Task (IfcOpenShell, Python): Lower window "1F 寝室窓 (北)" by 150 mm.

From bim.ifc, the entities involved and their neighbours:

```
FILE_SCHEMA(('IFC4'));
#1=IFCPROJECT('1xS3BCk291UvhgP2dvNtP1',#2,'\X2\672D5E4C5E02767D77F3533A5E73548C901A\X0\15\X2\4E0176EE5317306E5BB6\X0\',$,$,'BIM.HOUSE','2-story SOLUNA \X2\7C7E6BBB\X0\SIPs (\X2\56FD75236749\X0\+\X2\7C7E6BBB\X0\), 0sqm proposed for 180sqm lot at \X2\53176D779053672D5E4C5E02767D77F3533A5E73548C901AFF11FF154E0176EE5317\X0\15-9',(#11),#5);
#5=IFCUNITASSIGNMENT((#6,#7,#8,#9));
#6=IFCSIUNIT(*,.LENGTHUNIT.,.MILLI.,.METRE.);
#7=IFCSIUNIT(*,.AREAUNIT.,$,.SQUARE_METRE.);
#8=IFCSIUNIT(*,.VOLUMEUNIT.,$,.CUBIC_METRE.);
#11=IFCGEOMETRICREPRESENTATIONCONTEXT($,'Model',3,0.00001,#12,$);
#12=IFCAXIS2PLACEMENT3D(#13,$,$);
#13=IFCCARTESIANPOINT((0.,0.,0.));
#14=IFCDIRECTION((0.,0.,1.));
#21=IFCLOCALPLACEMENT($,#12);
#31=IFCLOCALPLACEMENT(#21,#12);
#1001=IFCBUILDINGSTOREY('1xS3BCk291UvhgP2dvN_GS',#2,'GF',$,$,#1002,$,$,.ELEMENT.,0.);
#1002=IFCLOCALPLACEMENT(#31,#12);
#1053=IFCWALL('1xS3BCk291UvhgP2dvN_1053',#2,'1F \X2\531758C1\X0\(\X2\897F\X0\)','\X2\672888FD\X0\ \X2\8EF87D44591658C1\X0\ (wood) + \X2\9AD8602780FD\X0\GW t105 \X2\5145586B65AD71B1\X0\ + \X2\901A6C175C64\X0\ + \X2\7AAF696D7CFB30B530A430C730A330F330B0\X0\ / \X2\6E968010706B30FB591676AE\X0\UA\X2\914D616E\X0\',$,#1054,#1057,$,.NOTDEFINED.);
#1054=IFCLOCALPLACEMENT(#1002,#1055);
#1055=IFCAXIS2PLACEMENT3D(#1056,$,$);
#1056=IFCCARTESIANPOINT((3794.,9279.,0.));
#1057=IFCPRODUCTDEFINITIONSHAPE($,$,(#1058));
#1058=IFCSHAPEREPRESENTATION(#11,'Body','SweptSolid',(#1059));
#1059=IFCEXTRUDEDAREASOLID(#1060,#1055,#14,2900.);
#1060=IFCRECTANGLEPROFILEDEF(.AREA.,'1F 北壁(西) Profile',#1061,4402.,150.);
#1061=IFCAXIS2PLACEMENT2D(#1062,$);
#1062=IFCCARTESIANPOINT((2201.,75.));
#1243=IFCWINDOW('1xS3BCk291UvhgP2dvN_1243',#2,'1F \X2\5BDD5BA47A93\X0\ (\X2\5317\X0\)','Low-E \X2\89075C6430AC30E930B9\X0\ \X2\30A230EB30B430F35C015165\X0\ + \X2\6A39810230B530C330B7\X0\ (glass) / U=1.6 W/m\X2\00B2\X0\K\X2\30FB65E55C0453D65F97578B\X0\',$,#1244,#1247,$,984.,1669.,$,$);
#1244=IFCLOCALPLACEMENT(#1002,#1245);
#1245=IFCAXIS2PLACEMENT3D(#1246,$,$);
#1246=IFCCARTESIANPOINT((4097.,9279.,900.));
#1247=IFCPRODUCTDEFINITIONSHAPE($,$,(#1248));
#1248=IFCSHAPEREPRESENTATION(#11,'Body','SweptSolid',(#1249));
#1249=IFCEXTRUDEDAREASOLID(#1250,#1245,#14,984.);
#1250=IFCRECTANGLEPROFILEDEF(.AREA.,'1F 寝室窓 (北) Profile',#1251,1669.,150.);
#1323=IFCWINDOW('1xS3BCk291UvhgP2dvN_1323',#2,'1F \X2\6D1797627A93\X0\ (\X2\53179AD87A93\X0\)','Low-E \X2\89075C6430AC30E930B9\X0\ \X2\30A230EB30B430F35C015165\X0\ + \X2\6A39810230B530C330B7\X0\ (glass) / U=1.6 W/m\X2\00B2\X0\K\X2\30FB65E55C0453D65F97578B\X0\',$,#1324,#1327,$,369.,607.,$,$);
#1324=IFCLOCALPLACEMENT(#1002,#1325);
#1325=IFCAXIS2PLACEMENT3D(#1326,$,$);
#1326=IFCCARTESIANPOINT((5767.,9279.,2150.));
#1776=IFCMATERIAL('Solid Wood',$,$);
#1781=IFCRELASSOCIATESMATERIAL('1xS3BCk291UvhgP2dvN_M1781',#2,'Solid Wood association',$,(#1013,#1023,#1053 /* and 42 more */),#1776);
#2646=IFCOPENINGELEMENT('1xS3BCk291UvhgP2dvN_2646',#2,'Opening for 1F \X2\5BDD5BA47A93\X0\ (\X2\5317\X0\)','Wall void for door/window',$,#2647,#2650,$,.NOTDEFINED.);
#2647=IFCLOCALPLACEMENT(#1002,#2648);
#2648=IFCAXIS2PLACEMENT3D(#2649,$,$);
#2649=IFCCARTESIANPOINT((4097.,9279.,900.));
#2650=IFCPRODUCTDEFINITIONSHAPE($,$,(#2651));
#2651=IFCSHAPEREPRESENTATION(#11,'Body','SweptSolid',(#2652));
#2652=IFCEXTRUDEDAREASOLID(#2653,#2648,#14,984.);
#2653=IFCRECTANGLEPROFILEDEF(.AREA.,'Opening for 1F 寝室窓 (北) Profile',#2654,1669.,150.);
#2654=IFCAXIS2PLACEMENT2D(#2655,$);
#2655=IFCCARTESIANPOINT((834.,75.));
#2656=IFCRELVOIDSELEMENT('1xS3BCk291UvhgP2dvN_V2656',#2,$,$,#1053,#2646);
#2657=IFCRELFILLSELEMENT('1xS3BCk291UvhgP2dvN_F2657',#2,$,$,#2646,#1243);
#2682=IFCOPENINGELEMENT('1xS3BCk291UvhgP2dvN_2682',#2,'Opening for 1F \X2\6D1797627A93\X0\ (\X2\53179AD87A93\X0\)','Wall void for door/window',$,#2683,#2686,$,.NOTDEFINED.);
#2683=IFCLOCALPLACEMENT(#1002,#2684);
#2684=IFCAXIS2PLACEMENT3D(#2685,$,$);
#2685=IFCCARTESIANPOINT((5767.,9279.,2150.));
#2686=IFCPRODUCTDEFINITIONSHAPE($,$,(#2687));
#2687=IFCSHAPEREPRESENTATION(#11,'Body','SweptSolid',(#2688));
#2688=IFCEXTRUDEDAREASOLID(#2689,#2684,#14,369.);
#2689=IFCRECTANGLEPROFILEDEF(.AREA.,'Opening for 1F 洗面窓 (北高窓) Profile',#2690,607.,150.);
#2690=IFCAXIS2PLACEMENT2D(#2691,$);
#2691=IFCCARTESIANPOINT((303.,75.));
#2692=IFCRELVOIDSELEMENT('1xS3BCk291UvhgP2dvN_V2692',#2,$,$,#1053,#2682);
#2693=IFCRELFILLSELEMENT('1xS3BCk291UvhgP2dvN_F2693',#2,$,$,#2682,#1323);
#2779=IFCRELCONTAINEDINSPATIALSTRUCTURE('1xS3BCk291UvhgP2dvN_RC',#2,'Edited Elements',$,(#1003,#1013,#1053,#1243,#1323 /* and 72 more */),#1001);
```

```python
import numpy as np
import ifcopenshell
import ifcopenshell.api.geometry
import ifcopenshell.util.placement
import ifcopenshell.util.unit

model = ifcopenshell.open("bim.ifc")
unit_scale = ifcopenshell.util.unit.calculate_unit_scale(model)

window = model.by_guid("1xS3BCk291UvhgP2dvN_1243")
opening = window.FillsVoids[0].RelatingOpeningElement
dz = -0.15 / unit_scale

shift = np.array([0.0, 0.0, dz])
# The window is not placed relative to its opening, so move both.
for product in (opening, window):
    matrix = ifcopenshell.util.placement.get_local_placement(product.ObjectPlacement)
    matrix[:3, 3] += shift
    ifcopenshell.api.geometry.edit_object_placement(model, product=product, matrix=matrix, is_si=False)

print(f"moved by {dz * unit_scale:+.3f} m")

model.write("bim_updated.ifc")
```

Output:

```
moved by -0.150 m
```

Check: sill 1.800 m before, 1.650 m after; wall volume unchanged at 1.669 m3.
